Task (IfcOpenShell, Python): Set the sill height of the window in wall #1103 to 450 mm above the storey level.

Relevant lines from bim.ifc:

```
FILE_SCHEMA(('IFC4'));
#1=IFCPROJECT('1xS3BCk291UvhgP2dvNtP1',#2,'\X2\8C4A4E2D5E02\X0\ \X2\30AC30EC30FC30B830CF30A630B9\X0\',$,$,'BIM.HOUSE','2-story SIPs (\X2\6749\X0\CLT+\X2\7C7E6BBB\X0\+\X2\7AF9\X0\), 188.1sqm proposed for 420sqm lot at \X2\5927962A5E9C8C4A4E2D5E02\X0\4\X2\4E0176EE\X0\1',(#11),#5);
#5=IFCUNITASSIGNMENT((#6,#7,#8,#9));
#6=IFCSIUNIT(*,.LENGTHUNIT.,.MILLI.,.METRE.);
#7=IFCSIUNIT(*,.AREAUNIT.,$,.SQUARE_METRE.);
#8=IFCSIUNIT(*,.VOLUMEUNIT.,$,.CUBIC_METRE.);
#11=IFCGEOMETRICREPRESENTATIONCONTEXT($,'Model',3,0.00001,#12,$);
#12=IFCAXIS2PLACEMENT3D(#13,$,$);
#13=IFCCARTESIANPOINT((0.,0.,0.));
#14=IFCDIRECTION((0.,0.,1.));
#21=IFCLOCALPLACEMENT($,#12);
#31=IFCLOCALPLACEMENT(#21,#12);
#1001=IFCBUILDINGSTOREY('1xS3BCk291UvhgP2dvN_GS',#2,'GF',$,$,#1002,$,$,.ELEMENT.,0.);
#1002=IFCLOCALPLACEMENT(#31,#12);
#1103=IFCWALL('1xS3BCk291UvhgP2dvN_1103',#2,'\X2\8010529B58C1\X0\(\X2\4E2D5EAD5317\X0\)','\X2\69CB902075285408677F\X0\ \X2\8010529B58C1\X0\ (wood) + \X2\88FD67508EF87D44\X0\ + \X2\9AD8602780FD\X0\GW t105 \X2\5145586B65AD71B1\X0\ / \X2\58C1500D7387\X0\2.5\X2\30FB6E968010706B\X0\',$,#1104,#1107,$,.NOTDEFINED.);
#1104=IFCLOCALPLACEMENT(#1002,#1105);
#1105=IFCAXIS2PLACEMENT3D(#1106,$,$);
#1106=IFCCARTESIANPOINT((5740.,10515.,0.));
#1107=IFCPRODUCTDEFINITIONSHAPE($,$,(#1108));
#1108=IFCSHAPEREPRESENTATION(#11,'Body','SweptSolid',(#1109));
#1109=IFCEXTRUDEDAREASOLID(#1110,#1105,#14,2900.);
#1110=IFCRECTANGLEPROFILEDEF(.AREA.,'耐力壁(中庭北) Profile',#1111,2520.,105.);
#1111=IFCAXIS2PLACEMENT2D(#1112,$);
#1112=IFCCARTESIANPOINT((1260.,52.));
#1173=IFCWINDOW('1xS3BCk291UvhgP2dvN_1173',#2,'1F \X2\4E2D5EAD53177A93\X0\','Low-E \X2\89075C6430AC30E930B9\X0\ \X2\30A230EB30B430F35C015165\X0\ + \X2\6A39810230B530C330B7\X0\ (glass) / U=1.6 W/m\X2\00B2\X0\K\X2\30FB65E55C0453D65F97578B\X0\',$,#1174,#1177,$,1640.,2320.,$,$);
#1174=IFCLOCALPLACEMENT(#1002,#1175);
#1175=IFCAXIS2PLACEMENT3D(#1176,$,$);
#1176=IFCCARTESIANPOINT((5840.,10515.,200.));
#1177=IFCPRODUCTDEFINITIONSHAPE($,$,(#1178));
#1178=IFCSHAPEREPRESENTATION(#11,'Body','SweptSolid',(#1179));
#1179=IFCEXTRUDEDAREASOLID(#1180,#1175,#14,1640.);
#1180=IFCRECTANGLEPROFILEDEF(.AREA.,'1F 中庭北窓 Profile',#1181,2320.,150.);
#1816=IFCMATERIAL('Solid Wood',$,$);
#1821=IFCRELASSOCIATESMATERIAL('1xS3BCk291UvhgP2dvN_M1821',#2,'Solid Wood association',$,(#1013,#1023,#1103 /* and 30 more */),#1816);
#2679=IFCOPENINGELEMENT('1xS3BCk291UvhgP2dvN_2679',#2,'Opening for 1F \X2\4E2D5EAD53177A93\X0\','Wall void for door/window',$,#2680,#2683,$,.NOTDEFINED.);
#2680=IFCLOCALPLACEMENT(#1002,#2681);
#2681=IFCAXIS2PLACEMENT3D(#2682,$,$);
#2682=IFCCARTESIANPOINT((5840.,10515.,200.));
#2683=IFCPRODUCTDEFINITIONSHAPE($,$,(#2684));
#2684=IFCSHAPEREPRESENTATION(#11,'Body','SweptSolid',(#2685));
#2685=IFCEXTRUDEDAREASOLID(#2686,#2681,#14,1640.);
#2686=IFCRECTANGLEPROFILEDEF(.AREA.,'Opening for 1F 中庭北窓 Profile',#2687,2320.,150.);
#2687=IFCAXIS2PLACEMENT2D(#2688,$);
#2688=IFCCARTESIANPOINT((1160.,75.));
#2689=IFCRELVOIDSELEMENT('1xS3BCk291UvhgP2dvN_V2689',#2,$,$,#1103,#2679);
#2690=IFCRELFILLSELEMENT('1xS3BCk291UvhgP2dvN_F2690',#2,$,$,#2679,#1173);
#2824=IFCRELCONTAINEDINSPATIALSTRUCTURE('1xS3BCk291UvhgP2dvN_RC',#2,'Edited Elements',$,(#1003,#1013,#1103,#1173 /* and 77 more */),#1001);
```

```python
import numpy as np
import ifcopenshell
import ifcopenshell.api.geometry
import ifcopenshell.geom
import ifcopenshell.util.element
import ifcopenshell.util.placement
import ifcopenshell.util.shape
import ifcopenshell.util.unit

model = ifcopenshell.open("bim.ifc")
unit_scale = ifcopenshell.util.unit.calculate_unit_scale(model)

window = model.by_guid("1xS3BCk291UvhgP2dvN_1173")
opening = window.FillsVoids[0].RelatingOpeningElement
storey = ifcopenshell.util.element.get_container(window, ifc_class="IfcBuildingStorey")
level = ifcopenshell.util.placement.get_local_placement(storey.ObjectPlacement)[2, 3]

# The opening's origin need not be at the sill, so measure its lowest point.
shape = ifcopenshell.geom.create_shape(ifcopenshell.geom.settings(), opening)
bottom = ifcopenshell.util.shape.get_shape_bottom_elevation(shape, shape.geometry) / unit_scale
dz = level + 450.0 - bottom

shift = np.array([0.0, 0.0, dz])
# The window is not placed relative to its opening, so move both.
for product in (opening, window):
    matrix = ifcopenshell.util.placement.get_local_placement(product.ObjectPlacement)
    matrix[:3, 3] += shift
    ifcopenshell.api.geometry.edit_object_placement(model, product=product, matrix=matrix, is_si=False)

print(f"moved by {dz * unit_scale:+.3f} m")

model.write("bim_updated.ifc")
```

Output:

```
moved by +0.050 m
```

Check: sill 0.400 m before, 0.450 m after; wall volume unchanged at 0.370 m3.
